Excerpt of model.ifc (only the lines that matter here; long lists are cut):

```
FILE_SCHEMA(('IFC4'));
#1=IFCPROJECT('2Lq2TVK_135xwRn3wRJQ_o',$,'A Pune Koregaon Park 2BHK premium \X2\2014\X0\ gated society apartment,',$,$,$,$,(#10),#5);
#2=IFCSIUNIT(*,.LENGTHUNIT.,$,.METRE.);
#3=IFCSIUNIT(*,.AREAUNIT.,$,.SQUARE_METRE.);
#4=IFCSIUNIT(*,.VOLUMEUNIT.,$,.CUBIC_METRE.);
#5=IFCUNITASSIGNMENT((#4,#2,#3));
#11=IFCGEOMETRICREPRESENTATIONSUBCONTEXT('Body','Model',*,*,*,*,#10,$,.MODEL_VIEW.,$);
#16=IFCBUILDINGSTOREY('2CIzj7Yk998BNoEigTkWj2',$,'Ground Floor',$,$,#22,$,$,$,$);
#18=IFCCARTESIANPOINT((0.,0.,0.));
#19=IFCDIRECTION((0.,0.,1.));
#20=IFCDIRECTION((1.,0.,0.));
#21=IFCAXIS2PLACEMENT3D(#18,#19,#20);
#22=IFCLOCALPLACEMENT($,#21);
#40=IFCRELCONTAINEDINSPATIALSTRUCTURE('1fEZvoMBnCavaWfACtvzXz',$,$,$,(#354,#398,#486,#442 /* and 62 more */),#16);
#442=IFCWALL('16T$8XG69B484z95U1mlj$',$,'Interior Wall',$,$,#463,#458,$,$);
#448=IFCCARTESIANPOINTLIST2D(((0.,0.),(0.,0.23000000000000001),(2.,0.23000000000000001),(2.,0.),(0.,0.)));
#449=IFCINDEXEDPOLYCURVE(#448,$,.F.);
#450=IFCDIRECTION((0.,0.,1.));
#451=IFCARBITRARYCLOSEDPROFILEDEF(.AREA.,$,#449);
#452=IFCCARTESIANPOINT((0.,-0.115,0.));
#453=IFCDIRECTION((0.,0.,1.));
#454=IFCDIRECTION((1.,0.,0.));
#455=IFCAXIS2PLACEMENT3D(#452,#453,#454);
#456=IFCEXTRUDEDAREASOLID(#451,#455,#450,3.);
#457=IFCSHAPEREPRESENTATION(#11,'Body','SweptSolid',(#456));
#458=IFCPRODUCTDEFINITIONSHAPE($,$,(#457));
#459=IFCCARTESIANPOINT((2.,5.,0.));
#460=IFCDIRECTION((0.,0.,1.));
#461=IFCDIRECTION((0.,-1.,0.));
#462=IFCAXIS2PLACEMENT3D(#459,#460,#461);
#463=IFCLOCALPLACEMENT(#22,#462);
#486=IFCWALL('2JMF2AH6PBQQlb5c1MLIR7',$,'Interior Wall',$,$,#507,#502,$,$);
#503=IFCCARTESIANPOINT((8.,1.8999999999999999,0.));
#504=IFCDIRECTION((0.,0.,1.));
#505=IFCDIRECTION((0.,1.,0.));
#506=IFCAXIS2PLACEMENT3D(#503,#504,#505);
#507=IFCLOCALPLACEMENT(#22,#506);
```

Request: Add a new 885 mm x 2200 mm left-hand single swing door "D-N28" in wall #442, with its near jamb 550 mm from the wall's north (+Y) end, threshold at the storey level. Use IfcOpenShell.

```python
import numpy as np
import ifcopenshell
import ifcopenshell.api.feature
import ifcopenshell.api.geometry
import ifcopenshell.api.root
import ifcopenshell.api.spatial
import ifcopenshell.geom
import ifcopenshell.util.element
import ifcopenshell.util.placement
import ifcopenshell.util.representation
import ifcopenshell.util.shape
import ifcopenshell.util.unit

model = ifcopenshell.open("model.ifc")
unit_scale = ifcopenshell.util.unit.calculate_unit_scale(model)
settings = ifcopenshell.geom.settings()


def volume(element):
    """Net volume in cubic metres, openings subtracted."""
    shape = ifcopenshell.geom.create_shape(settings, element)
    return ifcopenshell.util.shape.get_volume(shape.geometry)


wall = model.by_id(442)
storey = ifcopenshell.util.element.get_container(wall, ifc_class="IfcBuildingStorey")
context = ifcopenshell.util.representation.get_context(model, "Model", "Body", "MODEL_VIEW")
before = volume(wall)

width, height, from_end, sill = 0.885, 2.2, 0.55, 0.0  # metres

# The wall runs along its own X axis, and the end named is its -X end.
wall_shape = ifcopenshell.geom.create_shape(settings, wall)
x, y, z = ifcopenshell.util.shape.get_vertices(wall_shape.geometry).T
start = x.min() + from_end
face, thickness = float(y.min()), float(y.max() - y.min())
wall_matrix = ifcopenshell.util.placement.get_local_placement(wall.ObjectPlacement)
level = ifcopenshell.util.placement.get_local_placement(storey.ObjectPlacement)[2, 3]


def in_wall(x, y):
    """Placement at x, y metres in the wall's axes, at sill height."""
    matrix = wall_matrix.copy()
    matrix[:, 3] = wall_matrix @ np.array([x / unit_scale, y / unit_scale, 0.0, 1.0])
    matrix[2, 3] = level + sill / unit_scale
    return matrix


# Opening: a box that overshoots both wall faces by 50 mm.
opening = ifcopenshell.api.root.create_entity(model, ifc_class="IfcOpeningElement", predefined_type="OPENING")
box = ifcopenshell.api.geometry.add_wall_representation(
    model, context=context, length=width, height=height, thickness=thickness + 0.1
)
ifcopenshell.api.geometry.assign_representation(model, product=opening, representation=box)
ifcopenshell.api.geometry.edit_object_placement(model, product=opening, matrix=in_wall(start, face - 0.05), is_si=False)
ifcopenshell.api.feature.add_feature(model, feature=opening, element=wall)

door = ifcopenshell.api.root.create_entity(model, ifc_class="IfcDoor", name="D-N28", predefined_type="DOOR")
door.OverallWidth, door.OverallHeight = width / unit_scale, height / unit_scale
door.OperationType = "SINGLE_SWING_LEFT"
body = ifcopenshell.api.geometry.add_door_representation(
    model,
    context=context,
    overall_width=door.OverallWidth,
    overall_height=door.OverallHeight,
    operation_type="SINGLE_SWING_LEFT",
    lining_properties={"LiningDepth": thickness / unit_scale, "ThresholdDepth": thickness / unit_scale},
)
ifcopenshell.api.geometry.assign_representation(model, product=door, representation=body)
ifcopenshell.api.spatial.assign_container(model, products=[door], relating_structure=storey)
ifcopenshell.api.feature.add_filling(model, opening=opening, element=door)

# The lining spans the wall, so the door starts at the wall face.
ifcopenshell.api.geometry.edit_object_placement(model, product=door, matrix=in_wall(start, face), is_si=False)

after = volume(wall)

print(f"wall volume {before:.3f} -> {after:.3f} m3")

model.write("model_updated.ifc")
```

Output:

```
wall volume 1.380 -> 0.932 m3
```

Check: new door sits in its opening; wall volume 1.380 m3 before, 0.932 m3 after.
